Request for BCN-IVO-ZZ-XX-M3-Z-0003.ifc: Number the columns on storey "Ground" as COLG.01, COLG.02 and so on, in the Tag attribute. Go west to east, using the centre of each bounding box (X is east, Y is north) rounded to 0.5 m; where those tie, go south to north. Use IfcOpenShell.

First a look at what the model holds.

```python
import ifcopenshell
import ifcopenshell.util.element
import ifcopenshell.util.placement

model = ifcopenshell.open("BCN-IVO-ZZ-XX-M3-Z-0003.ifc")
print(model.schema)
storey = next(s for s in model.by_type("IfcBuildingStorey") if s.Name == "Ground")
columns = [e for e in ifcopenshell.util.element.get_decomposition(storey) if e.is_a("IfcColumn")]
for e in sorted(columns, key=lambda e: e.id()):
    origin = ifcopenshell.util.placement.get_local_placement(e.ObjectPlacement)[:3, 3]
    print(e.id(), e.Tag, e.Name, origin.round(2) + 0.0, sep=" | ")
```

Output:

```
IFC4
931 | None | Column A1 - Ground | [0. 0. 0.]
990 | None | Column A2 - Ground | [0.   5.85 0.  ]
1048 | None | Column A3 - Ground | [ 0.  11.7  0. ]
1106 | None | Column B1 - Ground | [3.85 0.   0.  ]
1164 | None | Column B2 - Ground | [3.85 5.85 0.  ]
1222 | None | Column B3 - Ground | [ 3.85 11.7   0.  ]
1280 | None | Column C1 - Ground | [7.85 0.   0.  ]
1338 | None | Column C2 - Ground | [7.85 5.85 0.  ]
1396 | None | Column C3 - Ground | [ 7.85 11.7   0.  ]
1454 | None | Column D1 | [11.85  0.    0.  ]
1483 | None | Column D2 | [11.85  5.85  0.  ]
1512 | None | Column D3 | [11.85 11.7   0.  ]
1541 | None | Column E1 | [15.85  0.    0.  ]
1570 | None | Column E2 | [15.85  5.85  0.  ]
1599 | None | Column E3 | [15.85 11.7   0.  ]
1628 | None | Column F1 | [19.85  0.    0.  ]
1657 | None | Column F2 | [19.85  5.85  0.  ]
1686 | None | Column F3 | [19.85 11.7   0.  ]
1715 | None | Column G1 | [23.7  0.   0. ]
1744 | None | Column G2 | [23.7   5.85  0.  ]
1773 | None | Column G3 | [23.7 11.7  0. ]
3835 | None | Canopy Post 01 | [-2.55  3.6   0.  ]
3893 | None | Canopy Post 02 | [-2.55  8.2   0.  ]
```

```python
import ifcopenshell
import ifcopenshell.geom
import ifcopenshell.util.element
import ifcopenshell.util.shape

model = ifcopenshell.open("BCN-IVO-ZZ-XX-M3-Z-0003.ifc")
settings = ifcopenshell.geom.settings()
settings.set("use-world-coords", True)


def centre(element):
    shape = ifcopenshell.geom.create_shape(settings, element)
    return ifcopenshell.util.shape.get_bbox_centroid(shape.geometry)


storey = next(s for s in model.by_type("IfcBuildingStorey") if s.Name == "Ground")
columns = [e for e in ifcopenshell.util.element.get_decomposition(storey) if e.is_a("IfcColumn")]

# Insertion points can sit at a corner or the storey origin, so sort by the geometry (in metres).
centres = {e: centre(e) for e in columns}
columns.sort(key=lambda e: (round(centres[e][0] / 0.5), centres[e][1]))

for i, e in enumerate(columns, start=1):
    number = f"COLG.{i:02d}"
    e.Tag = number
    print(e.id(), number)

model.write("BCN-IVO-ZZ-XX-M3-Z-0003_edited.ifc")
```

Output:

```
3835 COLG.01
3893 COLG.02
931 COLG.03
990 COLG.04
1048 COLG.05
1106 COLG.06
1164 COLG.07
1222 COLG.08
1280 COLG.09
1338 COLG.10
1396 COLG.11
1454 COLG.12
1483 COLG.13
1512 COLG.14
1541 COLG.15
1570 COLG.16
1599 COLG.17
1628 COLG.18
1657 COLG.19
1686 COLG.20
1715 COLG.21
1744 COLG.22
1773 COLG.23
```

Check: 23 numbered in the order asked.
